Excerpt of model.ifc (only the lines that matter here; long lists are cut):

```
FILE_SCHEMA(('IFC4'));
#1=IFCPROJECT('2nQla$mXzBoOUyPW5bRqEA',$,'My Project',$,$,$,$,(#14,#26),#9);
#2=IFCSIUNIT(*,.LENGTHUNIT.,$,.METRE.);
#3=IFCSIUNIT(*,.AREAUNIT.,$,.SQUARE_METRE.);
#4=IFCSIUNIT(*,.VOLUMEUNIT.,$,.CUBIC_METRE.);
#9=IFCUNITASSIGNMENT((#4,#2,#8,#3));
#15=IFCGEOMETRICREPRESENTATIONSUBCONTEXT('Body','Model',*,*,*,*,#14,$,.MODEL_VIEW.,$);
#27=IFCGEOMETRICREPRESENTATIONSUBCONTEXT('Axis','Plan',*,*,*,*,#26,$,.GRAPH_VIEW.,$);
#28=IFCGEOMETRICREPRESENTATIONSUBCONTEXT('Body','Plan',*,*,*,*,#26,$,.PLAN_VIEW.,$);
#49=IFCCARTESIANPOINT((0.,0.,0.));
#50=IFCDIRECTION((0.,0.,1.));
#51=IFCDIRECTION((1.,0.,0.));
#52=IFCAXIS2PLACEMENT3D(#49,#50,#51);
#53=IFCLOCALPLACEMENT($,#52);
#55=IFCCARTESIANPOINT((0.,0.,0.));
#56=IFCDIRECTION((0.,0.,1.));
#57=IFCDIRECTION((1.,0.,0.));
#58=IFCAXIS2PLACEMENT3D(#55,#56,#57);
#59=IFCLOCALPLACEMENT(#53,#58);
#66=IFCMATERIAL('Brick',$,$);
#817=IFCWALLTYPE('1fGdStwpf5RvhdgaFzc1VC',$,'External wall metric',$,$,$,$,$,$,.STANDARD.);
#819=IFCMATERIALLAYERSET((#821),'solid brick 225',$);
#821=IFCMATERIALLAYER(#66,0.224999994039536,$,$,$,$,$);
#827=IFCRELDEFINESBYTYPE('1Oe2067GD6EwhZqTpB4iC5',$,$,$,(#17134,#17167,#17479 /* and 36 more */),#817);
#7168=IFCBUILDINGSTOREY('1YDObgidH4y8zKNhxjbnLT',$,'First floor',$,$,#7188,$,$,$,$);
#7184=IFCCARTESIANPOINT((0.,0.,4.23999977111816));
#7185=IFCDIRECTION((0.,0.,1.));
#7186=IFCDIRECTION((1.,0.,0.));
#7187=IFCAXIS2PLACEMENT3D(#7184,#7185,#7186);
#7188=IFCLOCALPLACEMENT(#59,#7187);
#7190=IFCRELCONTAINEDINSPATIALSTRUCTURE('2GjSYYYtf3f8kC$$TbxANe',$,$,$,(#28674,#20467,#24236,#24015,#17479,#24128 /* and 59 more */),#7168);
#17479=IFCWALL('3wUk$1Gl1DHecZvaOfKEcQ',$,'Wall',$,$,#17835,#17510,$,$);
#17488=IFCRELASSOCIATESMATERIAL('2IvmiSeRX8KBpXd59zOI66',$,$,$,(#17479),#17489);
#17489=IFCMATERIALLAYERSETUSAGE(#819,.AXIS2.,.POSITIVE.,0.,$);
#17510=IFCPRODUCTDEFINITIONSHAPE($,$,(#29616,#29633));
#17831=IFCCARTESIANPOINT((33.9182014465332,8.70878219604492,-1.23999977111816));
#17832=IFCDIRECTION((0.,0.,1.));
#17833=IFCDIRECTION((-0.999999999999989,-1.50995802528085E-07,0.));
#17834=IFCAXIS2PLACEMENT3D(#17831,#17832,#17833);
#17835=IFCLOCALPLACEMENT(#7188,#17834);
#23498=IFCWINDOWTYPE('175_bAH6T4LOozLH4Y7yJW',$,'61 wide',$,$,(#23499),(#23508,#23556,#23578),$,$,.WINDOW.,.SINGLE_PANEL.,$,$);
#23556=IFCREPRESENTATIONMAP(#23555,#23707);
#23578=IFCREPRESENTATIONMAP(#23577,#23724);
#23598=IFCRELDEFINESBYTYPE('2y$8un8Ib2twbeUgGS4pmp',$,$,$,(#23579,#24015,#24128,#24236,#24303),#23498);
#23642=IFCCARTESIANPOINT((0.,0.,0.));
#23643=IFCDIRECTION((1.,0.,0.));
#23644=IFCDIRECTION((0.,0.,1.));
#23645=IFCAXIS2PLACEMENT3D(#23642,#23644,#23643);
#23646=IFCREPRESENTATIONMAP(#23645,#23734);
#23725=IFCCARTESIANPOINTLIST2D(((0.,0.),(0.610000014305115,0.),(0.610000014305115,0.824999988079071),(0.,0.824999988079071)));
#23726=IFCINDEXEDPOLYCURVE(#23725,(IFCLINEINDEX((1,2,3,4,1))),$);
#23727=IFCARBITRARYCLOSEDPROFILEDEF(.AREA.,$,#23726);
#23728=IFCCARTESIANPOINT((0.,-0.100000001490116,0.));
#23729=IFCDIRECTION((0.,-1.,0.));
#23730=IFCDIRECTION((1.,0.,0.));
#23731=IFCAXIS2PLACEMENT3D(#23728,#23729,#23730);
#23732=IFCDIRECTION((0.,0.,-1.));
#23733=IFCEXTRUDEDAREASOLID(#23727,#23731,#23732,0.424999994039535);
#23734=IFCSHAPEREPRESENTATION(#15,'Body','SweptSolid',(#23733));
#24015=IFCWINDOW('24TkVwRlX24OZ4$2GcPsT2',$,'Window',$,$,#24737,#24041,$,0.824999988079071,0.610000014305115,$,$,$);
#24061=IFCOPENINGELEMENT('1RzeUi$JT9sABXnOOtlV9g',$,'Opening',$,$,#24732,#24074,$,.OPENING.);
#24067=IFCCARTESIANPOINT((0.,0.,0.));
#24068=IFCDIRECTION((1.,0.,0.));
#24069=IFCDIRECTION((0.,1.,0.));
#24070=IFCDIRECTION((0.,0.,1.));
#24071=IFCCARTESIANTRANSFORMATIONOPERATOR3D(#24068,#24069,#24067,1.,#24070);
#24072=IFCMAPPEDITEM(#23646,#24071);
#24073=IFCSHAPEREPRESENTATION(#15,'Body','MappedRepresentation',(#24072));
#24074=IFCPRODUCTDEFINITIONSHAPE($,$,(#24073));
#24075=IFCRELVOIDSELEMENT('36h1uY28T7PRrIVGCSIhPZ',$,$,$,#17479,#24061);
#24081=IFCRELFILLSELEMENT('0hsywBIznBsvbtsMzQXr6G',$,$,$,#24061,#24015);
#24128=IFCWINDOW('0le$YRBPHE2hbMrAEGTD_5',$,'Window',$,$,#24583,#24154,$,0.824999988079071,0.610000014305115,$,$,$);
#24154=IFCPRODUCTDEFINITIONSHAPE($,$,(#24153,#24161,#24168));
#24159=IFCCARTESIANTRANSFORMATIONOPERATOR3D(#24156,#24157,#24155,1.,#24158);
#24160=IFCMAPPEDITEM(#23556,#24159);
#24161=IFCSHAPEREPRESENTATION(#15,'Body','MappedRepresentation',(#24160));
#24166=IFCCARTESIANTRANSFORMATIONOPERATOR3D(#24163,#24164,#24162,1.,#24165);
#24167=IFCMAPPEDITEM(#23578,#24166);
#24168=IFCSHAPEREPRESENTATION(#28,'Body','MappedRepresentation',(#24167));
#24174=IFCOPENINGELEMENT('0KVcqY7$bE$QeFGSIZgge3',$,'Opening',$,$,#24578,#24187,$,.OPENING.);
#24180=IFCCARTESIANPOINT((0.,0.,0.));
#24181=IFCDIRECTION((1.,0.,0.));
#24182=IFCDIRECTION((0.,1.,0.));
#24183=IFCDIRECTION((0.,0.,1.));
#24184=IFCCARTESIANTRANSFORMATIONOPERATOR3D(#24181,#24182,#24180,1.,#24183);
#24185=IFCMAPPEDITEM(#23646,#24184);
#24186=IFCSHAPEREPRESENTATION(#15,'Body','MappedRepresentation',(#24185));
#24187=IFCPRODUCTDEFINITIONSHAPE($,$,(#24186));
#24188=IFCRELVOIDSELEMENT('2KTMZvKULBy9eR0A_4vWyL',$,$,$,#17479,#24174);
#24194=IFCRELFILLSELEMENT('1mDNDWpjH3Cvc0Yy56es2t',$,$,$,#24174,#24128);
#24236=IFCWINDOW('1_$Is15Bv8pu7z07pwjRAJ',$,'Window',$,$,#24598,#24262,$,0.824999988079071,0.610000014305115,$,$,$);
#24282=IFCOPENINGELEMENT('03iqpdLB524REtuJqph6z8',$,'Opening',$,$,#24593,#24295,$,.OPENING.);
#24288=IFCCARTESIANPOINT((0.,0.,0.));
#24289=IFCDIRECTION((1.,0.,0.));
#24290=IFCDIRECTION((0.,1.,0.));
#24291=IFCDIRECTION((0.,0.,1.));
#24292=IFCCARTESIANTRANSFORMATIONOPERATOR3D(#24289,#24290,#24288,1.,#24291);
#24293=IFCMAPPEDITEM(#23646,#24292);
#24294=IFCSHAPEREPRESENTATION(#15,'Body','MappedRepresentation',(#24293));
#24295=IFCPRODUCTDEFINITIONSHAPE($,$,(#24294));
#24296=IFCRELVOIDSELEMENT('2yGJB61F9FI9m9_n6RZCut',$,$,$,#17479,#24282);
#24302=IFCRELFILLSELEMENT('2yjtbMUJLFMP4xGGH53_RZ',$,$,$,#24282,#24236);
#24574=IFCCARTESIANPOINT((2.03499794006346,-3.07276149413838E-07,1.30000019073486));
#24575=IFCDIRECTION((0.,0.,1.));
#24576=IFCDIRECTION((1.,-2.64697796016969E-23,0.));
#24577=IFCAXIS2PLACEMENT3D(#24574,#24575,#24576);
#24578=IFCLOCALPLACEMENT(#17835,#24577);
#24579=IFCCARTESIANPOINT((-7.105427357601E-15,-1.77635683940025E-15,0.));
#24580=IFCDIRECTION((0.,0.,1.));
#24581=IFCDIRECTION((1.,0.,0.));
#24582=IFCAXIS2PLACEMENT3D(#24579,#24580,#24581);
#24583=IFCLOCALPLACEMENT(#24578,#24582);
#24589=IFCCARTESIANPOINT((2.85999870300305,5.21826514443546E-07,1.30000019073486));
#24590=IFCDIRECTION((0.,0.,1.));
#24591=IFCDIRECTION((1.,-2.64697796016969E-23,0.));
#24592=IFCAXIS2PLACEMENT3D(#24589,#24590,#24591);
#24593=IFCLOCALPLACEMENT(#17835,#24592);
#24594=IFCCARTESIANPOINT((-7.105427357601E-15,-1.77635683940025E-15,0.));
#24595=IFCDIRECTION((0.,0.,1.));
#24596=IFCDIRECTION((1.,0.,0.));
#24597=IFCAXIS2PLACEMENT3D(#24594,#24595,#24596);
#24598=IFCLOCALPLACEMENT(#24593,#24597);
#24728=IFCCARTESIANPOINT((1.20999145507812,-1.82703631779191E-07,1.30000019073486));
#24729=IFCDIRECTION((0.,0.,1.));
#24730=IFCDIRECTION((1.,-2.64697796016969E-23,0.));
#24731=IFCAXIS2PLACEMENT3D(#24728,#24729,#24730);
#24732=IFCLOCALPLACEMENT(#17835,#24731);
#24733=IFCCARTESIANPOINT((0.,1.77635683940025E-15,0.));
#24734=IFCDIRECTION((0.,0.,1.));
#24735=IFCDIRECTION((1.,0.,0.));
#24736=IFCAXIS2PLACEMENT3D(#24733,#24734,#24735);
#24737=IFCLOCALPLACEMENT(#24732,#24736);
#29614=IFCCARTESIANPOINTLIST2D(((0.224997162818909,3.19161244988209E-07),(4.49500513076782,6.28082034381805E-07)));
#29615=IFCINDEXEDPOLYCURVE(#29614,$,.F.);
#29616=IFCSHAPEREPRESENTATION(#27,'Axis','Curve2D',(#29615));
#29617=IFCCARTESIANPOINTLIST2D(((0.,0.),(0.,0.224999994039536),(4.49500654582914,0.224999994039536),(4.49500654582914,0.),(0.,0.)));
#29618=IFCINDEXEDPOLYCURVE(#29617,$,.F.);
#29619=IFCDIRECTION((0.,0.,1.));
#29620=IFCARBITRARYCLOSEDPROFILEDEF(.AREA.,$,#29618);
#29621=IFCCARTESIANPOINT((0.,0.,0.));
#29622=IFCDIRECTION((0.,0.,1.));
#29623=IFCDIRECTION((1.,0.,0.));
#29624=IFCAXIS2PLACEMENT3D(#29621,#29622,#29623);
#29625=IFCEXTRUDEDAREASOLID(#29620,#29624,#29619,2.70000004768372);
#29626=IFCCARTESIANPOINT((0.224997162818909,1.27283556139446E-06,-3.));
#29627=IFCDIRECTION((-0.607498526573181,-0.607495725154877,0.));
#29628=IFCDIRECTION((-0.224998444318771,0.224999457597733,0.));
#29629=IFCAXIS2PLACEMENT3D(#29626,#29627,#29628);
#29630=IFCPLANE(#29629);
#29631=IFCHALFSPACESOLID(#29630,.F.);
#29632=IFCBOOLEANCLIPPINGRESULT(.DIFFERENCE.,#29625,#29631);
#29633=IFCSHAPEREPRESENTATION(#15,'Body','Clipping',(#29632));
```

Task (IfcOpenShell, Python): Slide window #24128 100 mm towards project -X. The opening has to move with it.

```python
import ifcopenshell
import ifcopenshell.api.geometry
import ifcopenshell.util.placement

model = ifcopenshell.open("model.ifc")

window = model.by_guid("0le$YRBPHE2hbMrAEGTD_5")
opening = window.FillsVoids[0].RelatingOpeningElement
wall = opening.VoidsElements[0].RelatingBuildingElement

wall_matrix = ifcopenshell.util.placement.get_local_placement(wall.ObjectPlacement)
shift = wall_matrix[:3, 0] * 0.1
before = ifcopenshell.util.placement.get_local_placement(window.ObjectPlacement)[:3, 3].copy()

# The window is placed relative to its opening, so it follows when the opening moves.
matrix = ifcopenshell.util.placement.get_local_placement(opening.ObjectPlacement)
matrix[:3, 3] += shift
ifcopenshell.api.geometry.edit_object_placement(
    model, product=opening, matrix=matrix, is_si=False, should_transform_children=True
)

after = ifcopenshell.util.placement.get_local_placement(window.ObjectPlacement)[:3, 3]
print("window moved by", (after - before).round(3) + 0.0)

model.write("model-out.ifc")
```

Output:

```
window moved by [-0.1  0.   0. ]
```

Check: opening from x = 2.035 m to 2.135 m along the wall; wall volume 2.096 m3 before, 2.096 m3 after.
